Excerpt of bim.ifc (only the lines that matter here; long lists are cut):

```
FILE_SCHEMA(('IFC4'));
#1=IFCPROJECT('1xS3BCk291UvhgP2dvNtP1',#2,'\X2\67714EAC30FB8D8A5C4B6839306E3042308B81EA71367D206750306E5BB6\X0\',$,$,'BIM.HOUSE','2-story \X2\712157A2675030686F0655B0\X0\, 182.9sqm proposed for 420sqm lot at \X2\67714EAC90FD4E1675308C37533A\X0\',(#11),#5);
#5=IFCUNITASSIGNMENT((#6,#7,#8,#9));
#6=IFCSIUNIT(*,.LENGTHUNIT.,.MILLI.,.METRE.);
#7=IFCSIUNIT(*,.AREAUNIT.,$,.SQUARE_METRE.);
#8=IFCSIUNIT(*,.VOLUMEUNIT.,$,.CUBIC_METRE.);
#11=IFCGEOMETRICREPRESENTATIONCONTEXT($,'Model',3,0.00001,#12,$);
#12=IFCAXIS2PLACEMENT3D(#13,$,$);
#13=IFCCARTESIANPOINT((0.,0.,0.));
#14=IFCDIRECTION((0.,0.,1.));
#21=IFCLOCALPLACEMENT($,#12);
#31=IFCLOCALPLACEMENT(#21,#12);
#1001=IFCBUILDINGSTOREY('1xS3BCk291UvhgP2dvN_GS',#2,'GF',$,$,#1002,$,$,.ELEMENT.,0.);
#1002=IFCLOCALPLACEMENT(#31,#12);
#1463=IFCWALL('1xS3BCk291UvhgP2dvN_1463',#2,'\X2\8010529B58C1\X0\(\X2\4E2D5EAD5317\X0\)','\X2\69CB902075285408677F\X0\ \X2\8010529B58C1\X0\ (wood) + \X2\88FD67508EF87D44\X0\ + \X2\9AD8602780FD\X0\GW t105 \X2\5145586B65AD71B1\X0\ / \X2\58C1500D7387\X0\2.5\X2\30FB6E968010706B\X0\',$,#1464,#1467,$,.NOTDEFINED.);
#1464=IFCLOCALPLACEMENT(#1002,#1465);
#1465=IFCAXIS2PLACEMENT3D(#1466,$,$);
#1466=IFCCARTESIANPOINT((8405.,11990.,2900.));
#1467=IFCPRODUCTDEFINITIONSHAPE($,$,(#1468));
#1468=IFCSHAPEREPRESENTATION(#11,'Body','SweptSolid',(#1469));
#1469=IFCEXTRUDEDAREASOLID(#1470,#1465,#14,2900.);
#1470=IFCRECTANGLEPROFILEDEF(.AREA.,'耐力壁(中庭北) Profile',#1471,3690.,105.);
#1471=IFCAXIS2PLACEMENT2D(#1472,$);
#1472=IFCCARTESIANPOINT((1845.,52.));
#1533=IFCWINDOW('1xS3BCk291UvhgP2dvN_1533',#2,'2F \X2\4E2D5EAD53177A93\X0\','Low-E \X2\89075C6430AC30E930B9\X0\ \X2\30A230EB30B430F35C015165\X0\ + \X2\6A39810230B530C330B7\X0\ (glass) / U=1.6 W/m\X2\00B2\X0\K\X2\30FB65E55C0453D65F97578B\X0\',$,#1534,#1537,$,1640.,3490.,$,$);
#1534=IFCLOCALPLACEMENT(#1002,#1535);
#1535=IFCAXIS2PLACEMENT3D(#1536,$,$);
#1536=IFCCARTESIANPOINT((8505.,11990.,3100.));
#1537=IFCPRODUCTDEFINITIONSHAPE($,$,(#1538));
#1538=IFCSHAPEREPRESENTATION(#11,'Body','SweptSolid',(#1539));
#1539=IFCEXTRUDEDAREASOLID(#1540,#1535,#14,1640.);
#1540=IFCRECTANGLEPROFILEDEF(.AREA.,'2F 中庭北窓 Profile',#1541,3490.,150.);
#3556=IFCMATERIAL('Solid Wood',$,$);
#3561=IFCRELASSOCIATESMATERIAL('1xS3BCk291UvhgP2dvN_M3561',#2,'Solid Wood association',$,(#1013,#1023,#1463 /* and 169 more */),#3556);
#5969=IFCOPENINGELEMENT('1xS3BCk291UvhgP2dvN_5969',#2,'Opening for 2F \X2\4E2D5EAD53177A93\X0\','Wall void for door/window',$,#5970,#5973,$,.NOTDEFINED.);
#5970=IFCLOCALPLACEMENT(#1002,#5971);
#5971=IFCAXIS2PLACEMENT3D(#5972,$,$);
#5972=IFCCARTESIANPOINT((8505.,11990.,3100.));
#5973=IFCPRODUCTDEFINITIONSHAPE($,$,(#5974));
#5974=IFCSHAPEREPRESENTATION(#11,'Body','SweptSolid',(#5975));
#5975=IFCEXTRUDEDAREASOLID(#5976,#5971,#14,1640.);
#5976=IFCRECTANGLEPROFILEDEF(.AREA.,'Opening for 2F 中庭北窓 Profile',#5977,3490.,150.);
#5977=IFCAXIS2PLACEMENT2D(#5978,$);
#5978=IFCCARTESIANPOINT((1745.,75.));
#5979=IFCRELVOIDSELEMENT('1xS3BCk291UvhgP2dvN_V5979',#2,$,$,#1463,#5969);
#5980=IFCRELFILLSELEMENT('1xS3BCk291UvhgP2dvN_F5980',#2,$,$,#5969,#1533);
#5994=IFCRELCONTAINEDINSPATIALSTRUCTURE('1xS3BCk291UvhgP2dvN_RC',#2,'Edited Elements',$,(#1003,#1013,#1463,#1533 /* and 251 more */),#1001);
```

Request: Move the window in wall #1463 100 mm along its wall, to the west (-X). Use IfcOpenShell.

```python
import ifcopenshell
import ifcopenshell.api.geometry
import ifcopenshell.util.placement
import ifcopenshell.util.unit

model = ifcopenshell.open("bim.ifc")
unit_scale = ifcopenshell.util.unit.calculate_unit_scale(model)

window = model.by_guid("1xS3BCk291UvhgP2dvN_1533")
opening = window.FillsVoids[0].RelatingOpeningElement
wall = opening.VoidsElements[0].RelatingBuildingElement

wall_matrix = ifcopenshell.util.placement.get_local_placement(wall.ObjectPlacement)
shift = wall_matrix[:3, 0] * -0.1 / unit_scale
before = ifcopenshell.util.placement.get_local_placement(window.ObjectPlacement)[:3, 3].copy()

# The window is not placed relative to its opening, so move both.
for product in (opening, window):
    matrix = ifcopenshell.util.placement.get_local_placement(product.ObjectPlacement)
    matrix[:3, 3] += shift
    ifcopenshell.api.geometry.edit_object_placement(model, product=product, matrix=matrix, is_si=False)

after = ifcopenshell.util.placement.get_local_placement(window.ObjectPlacement)[:3, 3]
print("window moved by", (after - before).round(3) + 0.0)

model.write("bim_updated.ifc")
```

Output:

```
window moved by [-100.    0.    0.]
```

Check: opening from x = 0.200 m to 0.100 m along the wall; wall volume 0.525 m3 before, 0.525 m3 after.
